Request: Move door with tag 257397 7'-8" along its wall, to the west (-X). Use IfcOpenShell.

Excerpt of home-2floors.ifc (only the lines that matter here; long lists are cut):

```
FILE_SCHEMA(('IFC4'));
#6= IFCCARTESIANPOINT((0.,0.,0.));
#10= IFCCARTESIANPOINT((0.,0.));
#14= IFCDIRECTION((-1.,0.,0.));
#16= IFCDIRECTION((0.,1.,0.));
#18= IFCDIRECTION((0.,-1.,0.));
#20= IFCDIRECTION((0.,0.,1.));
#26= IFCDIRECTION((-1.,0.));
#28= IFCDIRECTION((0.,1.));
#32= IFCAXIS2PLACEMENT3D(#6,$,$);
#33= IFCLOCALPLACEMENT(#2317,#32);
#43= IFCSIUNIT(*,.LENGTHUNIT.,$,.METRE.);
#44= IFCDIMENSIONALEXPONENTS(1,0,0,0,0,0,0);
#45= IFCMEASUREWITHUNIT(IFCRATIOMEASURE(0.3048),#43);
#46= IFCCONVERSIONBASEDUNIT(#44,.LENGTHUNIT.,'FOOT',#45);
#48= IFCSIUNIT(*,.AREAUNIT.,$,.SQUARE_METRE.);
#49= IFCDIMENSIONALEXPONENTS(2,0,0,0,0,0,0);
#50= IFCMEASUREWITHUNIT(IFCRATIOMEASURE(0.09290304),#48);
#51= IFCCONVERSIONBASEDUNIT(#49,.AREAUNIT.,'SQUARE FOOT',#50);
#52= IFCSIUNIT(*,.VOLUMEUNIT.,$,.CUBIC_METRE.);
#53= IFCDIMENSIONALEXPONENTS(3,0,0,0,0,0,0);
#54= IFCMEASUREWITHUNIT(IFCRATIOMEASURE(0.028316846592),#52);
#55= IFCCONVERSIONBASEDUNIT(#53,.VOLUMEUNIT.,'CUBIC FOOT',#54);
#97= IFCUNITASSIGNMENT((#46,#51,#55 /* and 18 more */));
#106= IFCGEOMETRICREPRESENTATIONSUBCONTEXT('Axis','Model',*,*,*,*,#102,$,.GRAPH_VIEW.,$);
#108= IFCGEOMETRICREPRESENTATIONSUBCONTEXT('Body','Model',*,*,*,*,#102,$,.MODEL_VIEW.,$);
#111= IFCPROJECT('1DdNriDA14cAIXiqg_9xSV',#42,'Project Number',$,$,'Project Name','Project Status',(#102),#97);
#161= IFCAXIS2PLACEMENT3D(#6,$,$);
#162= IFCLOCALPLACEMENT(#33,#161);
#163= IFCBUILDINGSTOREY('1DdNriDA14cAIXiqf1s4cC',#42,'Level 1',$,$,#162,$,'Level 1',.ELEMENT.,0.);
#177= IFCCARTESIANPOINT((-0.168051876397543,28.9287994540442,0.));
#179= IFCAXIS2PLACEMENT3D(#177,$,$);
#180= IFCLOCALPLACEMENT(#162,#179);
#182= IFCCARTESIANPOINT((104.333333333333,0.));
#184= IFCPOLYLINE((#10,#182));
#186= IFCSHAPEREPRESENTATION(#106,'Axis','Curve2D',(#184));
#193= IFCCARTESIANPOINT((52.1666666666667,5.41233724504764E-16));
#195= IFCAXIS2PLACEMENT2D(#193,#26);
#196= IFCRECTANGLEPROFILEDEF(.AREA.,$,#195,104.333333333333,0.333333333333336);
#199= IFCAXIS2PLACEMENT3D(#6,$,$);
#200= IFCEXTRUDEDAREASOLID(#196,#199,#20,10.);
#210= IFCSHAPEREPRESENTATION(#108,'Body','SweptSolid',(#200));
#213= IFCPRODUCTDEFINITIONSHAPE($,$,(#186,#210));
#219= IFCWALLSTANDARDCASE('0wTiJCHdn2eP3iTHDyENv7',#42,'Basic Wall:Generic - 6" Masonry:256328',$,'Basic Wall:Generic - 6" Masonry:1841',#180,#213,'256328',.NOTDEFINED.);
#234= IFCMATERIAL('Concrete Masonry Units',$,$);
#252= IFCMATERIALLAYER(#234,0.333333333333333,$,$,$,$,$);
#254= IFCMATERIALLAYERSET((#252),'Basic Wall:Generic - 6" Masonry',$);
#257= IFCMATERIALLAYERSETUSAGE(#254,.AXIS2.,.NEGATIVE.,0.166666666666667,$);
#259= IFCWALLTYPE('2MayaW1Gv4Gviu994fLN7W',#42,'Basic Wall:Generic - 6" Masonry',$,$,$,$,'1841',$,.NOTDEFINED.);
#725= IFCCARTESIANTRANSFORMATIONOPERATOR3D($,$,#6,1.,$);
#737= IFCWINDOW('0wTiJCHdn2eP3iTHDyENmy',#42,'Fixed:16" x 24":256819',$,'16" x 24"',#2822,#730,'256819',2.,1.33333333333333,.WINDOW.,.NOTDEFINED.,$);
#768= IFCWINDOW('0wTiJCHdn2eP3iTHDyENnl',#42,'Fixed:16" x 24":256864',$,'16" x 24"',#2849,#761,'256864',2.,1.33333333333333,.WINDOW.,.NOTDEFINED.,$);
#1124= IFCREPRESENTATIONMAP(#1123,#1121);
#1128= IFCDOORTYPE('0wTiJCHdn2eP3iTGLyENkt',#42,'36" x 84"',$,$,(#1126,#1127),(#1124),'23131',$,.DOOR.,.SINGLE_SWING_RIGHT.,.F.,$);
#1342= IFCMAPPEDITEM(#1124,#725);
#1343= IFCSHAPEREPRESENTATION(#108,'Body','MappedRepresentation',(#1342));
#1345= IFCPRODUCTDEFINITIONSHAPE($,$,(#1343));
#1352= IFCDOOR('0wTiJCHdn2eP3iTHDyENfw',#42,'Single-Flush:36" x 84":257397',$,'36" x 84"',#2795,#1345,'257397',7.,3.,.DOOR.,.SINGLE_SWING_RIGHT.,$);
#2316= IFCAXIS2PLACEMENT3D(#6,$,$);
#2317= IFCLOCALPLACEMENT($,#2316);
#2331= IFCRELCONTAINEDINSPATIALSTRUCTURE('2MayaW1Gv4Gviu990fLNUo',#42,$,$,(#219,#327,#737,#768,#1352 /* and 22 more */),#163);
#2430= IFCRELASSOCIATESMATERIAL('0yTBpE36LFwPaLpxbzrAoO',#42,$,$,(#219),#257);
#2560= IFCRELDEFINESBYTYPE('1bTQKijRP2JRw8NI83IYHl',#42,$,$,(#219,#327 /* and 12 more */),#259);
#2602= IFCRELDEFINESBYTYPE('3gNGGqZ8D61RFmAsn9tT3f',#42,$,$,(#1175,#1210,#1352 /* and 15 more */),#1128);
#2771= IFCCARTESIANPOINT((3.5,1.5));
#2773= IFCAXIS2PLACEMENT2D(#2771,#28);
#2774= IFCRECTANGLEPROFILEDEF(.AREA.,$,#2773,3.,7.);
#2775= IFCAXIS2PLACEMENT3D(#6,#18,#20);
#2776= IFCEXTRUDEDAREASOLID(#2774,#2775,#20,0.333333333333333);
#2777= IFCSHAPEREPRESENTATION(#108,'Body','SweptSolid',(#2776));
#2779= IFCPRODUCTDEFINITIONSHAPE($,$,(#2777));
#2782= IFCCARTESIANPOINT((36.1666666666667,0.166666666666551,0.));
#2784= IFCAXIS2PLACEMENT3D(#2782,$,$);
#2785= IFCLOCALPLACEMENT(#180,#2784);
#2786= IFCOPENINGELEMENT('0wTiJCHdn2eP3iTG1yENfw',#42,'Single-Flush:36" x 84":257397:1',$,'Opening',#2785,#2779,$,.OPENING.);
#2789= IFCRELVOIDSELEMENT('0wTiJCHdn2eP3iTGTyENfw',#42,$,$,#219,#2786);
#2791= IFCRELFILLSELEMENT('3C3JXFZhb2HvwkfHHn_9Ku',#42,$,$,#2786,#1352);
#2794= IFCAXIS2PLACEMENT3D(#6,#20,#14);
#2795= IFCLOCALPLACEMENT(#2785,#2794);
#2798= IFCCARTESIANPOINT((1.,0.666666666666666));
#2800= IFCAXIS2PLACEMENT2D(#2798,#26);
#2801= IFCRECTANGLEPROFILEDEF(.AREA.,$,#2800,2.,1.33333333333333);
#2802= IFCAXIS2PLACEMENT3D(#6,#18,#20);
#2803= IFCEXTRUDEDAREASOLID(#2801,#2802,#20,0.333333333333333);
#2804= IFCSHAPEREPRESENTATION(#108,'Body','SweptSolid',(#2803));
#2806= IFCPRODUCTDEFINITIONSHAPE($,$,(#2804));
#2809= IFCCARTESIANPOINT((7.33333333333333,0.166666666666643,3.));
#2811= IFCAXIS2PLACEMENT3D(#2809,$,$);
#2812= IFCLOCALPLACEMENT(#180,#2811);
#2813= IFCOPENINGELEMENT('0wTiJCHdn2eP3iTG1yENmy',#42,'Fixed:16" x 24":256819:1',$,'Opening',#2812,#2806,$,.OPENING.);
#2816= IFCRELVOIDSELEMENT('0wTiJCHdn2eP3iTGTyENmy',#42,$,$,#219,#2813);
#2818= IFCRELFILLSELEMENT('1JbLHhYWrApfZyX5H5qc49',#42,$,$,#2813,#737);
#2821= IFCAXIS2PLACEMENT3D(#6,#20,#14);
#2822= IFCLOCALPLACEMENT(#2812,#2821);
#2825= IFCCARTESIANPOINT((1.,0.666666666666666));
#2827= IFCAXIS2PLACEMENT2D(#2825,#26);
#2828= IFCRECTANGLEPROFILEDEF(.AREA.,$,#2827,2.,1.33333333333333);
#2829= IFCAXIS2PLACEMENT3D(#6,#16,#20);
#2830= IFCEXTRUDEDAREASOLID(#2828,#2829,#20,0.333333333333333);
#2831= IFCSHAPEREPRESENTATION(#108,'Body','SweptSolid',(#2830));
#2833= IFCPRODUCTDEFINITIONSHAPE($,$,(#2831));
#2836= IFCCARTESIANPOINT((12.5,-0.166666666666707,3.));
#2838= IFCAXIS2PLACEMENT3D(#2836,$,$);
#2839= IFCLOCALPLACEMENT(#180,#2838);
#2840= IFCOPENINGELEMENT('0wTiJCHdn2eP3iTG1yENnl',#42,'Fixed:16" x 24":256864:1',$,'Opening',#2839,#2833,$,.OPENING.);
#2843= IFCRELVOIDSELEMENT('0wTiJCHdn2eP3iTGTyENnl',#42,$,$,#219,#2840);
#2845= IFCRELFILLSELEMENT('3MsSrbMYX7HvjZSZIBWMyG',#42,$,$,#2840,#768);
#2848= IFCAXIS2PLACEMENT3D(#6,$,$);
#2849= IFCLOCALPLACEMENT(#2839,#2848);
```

```python
import ifcopenshell
import ifcopenshell.api.geometry
import ifcopenshell.util.placement
import ifcopenshell.util.unit

model = ifcopenshell.open("home-2floors.ifc")
unit_scale = ifcopenshell.util.unit.calculate_unit_scale(model)

door = model.by_guid("0wTiJCHdn2eP3iTHDyENfw")
opening = door.FillsVoids[0].RelatingOpeningElement
wall = opening.VoidsElements[0].RelatingBuildingElement

wall_matrix = ifcopenshell.util.placement.get_local_placement(wall.ObjectPlacement)
shift = wall_matrix[:3, 0] * -92 * 0.0254 / unit_scale
before = ifcopenshell.util.placement.get_local_placement(door.ObjectPlacement)[:3, 3].copy()

# The door is placed relative to its opening, so it follows when the opening moves.
matrix = ifcopenshell.util.placement.get_local_placement(opening.ObjectPlacement)
matrix[:3, 3] += shift
ifcopenshell.api.geometry.edit_object_placement(
    model, product=opening, matrix=matrix, is_si=False, should_transform_children=True
)

after = ifcopenshell.util.placement.get_local_placement(door.ObjectPlacement)[:3, 3]
print("door moved by", (after - before).round(3) + 0.0)

model.write("home-2floors_rev.ifc")
```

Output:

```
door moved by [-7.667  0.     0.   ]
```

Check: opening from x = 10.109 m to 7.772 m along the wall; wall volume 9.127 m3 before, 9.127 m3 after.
